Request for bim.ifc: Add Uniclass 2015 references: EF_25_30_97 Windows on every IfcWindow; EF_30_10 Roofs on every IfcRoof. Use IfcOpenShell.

First a look at what the model holds.

```python
import ifcopenshell

model = ifcopenshell.open("bim.ifc")
print(model.schema)
print("classifications:", [c.Name for c in model.by_type("IfcClassification")])
for ifc_class in ("IfcDoor", "IfcRoof", "IfcStair", "IfcWall", "IfcWindow"):
    print(ifc_class, len(model.by_type(ifc_class)))
```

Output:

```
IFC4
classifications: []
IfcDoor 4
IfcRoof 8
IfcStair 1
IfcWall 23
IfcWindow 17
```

```python
import ifcopenshell
import ifcopenshell.api.classification

model = ifcopenshell.open("bim.ifc")

system = ifcopenshell.api.classification.add_classification(model, classification="Uniclass 2015")

codes = {
    "IfcWindow": ("EF_25_30_97", "Windows"),
    "IfcRoof": ("EF_30_10", "Roofs"),
}
for ifc_class, (code, name) in codes.items():
    products = model.by_type(ifc_class)
    ifcopenshell.api.classification.add_reference(
        model, products=products, classification=system, identification=code, name=name
    )
    print(code, len(products))

model.write("bim_v2.ifc")
```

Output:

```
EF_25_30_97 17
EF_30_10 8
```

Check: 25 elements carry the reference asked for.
